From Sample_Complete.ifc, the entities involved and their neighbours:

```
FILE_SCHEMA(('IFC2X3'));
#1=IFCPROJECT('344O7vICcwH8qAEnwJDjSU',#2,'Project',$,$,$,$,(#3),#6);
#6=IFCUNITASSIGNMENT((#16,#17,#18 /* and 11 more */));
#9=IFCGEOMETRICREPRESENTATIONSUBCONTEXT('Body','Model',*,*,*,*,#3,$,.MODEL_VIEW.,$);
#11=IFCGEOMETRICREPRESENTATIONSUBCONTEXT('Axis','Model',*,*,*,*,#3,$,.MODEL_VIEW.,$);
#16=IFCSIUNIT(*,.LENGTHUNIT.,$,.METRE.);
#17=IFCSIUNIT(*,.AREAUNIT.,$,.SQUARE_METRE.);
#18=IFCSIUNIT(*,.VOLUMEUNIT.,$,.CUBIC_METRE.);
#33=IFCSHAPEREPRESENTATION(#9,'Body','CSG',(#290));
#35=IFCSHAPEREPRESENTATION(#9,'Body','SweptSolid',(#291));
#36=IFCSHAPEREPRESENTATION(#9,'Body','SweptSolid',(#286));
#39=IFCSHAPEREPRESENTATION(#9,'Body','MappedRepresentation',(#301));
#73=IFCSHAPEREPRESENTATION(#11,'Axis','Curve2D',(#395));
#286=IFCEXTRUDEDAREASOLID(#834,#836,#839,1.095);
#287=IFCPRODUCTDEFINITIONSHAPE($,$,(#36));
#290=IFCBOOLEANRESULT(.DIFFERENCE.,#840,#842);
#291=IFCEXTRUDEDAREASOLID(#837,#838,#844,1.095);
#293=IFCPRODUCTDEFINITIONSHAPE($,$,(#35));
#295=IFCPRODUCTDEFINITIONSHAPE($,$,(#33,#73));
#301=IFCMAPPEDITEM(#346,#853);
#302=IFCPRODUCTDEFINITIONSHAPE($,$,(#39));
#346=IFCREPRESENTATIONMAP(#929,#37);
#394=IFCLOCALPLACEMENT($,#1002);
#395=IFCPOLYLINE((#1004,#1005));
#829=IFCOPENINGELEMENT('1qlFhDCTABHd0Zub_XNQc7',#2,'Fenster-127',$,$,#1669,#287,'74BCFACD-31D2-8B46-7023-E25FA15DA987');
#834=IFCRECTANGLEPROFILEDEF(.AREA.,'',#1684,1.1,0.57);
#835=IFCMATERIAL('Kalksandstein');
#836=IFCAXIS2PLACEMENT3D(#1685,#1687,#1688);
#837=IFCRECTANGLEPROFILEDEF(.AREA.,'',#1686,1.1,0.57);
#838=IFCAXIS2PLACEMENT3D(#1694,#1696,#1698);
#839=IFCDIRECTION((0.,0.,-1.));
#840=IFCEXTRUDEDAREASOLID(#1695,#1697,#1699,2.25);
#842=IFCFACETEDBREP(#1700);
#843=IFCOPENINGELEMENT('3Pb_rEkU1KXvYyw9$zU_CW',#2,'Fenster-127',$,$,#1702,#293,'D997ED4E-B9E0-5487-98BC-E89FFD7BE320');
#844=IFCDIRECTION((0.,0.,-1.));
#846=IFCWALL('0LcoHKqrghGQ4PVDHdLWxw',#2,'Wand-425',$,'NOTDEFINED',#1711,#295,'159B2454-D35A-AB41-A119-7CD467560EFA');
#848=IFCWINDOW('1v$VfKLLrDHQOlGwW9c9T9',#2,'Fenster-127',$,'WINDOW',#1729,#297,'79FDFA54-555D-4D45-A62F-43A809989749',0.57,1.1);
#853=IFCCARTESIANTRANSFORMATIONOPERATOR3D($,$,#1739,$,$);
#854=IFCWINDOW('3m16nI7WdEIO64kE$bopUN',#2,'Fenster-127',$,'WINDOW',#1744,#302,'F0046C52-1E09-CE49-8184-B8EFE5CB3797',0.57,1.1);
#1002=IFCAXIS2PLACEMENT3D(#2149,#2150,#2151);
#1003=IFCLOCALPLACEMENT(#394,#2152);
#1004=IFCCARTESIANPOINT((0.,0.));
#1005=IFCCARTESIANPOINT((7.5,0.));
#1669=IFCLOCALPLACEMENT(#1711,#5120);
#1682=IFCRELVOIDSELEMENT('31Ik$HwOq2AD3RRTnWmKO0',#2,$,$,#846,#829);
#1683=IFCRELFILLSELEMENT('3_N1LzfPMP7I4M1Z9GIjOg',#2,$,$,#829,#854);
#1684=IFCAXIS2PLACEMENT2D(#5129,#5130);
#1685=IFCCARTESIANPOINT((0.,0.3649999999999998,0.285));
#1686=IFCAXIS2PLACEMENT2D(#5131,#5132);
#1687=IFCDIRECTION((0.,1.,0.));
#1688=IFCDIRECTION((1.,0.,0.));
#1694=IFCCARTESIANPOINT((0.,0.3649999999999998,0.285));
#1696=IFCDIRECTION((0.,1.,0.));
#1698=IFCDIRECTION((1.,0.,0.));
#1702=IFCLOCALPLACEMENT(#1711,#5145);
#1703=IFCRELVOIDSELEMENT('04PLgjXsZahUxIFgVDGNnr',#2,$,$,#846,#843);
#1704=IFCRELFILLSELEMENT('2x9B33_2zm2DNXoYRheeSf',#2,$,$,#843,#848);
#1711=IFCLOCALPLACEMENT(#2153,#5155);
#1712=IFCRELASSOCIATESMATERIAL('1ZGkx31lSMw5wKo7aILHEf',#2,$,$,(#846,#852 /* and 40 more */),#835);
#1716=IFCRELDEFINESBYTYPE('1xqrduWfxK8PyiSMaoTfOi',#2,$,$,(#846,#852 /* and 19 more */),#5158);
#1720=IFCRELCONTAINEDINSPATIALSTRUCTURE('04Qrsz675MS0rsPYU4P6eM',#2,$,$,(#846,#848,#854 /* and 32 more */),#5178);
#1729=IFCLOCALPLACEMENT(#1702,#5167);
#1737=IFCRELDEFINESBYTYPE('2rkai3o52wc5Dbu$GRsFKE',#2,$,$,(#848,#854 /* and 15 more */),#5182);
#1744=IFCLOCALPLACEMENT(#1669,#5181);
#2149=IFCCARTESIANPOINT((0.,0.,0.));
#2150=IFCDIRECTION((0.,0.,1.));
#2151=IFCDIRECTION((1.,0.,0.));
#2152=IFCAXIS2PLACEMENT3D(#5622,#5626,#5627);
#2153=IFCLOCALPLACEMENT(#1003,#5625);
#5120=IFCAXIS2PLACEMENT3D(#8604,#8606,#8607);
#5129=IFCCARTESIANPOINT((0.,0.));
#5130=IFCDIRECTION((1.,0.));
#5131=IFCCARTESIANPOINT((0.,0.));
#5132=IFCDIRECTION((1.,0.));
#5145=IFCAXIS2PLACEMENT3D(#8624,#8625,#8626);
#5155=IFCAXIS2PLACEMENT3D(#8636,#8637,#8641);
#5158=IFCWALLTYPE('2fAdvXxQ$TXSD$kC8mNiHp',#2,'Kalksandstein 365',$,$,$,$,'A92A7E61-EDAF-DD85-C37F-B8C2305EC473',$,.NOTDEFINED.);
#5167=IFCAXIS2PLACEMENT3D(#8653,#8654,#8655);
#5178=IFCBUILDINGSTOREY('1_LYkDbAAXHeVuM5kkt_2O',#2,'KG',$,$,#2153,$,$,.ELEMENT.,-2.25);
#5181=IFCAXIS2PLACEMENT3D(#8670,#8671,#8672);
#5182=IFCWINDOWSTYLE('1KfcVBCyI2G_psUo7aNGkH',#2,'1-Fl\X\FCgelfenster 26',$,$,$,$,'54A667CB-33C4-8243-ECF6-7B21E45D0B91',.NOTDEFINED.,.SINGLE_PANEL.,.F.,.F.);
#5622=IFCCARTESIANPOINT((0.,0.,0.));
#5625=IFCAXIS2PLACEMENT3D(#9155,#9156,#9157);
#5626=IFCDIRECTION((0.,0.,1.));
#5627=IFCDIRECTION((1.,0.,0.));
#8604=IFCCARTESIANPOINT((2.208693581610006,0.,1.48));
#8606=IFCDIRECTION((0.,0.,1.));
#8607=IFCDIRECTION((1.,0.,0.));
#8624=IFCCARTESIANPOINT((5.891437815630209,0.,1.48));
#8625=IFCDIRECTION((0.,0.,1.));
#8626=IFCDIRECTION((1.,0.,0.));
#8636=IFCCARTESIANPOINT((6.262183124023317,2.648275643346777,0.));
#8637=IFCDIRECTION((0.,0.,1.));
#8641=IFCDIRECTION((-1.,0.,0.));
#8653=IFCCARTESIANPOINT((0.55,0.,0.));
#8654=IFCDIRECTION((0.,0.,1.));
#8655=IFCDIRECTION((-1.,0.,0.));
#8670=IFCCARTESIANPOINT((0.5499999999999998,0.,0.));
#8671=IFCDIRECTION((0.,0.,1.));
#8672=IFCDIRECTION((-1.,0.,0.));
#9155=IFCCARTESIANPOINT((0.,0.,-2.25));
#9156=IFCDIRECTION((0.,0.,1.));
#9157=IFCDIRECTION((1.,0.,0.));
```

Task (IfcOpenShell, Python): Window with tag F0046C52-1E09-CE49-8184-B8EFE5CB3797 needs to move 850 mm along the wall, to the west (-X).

```python
import ifcopenshell
import ifcopenshell.api.geometry
import ifcopenshell.util.placement
import ifcopenshell.util.unit

model = ifcopenshell.open("Sample_Complete.ifc")
unit_scale = ifcopenshell.util.unit.calculate_unit_scale(model)

window = model.by_id(854)
opening = window.FillsVoids[0].RelatingOpeningElement
wall = opening.VoidsElements[0].RelatingBuildingElement

wall_matrix = ifcopenshell.util.placement.get_local_placement(wall.ObjectPlacement)
shift = wall_matrix[:3, 0] * 0.85 / unit_scale
before = ifcopenshell.util.placement.get_local_placement(window.ObjectPlacement)[:3, 3].copy()

# The window is placed relative to its opening, so it follows when the opening moves.
matrix = ifcopenshell.util.placement.get_local_placement(opening.ObjectPlacement)
matrix[:3, 3] += shift
ifcopenshell.api.geometry.edit_object_placement(
    model, product=opening, matrix=matrix, is_si=False, should_transform_children=True
)

after = ifcopenshell.util.placement.get_local_placement(window.ObjectPlacement)[:3, 3]
print("window moved by", (after - before).round(3) + 0.0)

model.write("Sample_Complete-out.ifc")
```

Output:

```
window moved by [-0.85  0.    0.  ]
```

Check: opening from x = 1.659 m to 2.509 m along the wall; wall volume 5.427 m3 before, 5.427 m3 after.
